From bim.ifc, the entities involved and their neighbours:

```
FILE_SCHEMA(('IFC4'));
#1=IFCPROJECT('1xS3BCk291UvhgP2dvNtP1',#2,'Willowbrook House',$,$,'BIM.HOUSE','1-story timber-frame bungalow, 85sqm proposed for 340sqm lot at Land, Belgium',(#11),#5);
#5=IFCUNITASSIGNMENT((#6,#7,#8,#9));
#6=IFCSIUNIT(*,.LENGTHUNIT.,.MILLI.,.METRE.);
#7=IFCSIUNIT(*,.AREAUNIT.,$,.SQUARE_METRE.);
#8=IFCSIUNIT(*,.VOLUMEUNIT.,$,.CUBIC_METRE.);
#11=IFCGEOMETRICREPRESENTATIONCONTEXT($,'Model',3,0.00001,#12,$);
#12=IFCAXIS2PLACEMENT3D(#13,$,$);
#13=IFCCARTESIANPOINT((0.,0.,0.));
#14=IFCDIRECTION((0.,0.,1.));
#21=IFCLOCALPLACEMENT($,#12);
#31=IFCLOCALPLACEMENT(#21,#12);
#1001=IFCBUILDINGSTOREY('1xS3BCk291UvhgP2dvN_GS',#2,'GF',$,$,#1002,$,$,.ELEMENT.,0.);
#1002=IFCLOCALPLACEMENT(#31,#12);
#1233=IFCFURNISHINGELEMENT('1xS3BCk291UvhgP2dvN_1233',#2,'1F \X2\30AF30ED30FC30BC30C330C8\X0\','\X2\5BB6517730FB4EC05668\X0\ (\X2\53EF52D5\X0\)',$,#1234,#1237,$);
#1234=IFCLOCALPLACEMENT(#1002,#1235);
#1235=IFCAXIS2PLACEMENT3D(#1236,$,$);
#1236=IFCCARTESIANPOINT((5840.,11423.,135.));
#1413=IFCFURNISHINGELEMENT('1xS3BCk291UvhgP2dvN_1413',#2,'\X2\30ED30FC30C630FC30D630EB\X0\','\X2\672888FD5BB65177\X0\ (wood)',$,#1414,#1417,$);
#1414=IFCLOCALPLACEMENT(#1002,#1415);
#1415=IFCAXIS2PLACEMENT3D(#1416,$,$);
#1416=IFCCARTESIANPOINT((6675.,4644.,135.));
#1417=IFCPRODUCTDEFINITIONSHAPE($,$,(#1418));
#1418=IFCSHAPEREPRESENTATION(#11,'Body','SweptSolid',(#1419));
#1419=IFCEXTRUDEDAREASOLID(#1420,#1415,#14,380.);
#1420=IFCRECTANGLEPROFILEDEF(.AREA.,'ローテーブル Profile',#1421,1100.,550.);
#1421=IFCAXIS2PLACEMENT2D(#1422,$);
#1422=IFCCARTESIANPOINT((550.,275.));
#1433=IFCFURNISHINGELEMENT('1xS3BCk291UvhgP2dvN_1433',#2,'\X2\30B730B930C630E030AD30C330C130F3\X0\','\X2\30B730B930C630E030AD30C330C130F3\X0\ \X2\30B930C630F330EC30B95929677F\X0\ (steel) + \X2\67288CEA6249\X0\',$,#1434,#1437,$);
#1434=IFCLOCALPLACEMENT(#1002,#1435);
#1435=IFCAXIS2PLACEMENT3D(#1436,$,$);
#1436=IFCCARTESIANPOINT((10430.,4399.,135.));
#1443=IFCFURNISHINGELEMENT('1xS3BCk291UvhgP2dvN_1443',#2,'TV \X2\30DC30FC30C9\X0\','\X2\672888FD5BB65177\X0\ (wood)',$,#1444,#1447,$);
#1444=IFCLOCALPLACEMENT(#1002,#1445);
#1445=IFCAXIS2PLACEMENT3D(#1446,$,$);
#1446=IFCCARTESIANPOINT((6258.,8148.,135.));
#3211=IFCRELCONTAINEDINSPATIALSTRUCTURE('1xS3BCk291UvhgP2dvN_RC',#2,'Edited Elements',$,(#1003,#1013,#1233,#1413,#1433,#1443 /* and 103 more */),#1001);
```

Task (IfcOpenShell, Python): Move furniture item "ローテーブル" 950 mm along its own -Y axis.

```python
import ifcopenshell
import ifcopenshell.api.geometry
import ifcopenshell.util.placement
import ifcopenshell.util.unit

model = ifcopenshell.open("bim.ifc")
unit_scale = ifcopenshell.util.unit.calculate_unit_scale(model)

item = model.by_id(1413)
matrix = ifcopenshell.util.placement.get_local_placement(item.ObjectPlacement)
matrix[:3, 3] -= matrix[:3, 1] * 0.95 / unit_scale
ifcopenshell.api.geometry.edit_object_placement(model, product=item, matrix=matrix, is_si=False)

print(ifcopenshell.util.placement.get_local_placement(item.ObjectPlacement).round(3) + 0.0)

model.write("bim_updated.ifc")
```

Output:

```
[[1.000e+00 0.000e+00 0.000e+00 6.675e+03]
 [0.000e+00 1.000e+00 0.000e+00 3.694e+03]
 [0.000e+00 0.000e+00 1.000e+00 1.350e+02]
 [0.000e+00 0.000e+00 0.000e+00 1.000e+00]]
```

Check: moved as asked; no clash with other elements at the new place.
